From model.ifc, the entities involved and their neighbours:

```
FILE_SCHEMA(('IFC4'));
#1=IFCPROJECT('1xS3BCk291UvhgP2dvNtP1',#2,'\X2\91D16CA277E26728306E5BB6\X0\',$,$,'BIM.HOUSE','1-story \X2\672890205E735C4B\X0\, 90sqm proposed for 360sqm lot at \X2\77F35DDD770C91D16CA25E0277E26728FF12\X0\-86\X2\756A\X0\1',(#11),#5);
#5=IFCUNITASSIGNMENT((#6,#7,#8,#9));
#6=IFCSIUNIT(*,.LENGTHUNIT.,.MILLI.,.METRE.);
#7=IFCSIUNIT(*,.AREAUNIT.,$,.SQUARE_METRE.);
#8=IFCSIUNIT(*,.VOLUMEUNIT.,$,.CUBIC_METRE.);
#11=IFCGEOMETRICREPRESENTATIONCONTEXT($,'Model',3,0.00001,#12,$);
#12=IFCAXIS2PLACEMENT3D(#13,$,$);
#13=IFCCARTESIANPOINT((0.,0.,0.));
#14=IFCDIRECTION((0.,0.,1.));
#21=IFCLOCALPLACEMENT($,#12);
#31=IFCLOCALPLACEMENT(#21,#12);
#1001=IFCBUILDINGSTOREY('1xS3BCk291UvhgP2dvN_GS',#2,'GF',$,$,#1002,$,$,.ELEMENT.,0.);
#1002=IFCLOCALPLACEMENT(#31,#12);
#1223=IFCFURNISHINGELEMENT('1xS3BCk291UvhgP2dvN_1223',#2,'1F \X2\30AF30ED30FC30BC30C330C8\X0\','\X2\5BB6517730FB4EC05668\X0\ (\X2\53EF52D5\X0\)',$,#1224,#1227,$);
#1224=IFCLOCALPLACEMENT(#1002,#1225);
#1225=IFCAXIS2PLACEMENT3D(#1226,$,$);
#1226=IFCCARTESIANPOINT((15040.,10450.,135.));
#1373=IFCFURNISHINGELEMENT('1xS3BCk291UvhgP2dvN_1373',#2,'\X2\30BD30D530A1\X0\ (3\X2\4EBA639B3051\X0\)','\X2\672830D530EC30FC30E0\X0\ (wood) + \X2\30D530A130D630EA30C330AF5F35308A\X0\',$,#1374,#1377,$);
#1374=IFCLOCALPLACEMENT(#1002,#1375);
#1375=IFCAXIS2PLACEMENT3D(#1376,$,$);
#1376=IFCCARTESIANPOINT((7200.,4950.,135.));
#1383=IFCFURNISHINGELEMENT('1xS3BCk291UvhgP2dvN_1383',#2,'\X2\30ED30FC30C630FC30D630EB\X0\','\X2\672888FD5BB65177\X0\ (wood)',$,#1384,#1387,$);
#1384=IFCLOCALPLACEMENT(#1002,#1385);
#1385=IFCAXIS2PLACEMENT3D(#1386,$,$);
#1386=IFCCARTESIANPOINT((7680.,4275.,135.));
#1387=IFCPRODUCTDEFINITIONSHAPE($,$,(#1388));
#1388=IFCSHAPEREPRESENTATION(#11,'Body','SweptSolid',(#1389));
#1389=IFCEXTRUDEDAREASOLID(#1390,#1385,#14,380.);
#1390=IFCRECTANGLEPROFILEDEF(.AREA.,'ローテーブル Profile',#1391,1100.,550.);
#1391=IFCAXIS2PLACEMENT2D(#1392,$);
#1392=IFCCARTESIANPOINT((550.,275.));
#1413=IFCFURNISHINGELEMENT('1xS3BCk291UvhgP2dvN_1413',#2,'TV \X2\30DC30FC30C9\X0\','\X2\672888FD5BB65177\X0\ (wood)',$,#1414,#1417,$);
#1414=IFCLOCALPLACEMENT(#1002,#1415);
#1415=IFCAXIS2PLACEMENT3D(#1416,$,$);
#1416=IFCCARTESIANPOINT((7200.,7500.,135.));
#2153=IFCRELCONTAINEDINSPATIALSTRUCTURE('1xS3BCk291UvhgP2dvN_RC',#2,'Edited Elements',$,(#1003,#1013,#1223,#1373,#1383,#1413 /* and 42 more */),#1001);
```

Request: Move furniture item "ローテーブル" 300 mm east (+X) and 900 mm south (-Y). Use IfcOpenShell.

```python
import ifcopenshell
import ifcopenshell.api.geometry
import ifcopenshell.util.placement

model = ifcopenshell.open("model.ifc")

item = model.by_guid("1xS3BCk291UvhgP2dvN_1383")
matrix = ifcopenshell.util.placement.get_local_placement(item.ObjectPlacement)
matrix[0, 3] += 300.0
matrix[1, 3] -= 900.0
ifcopenshell.api.geometry.edit_object_placement(model, product=item, matrix=matrix, is_si=False)

print(ifcopenshell.util.placement.get_local_placement(item.ObjectPlacement).round(3) + 0.0)

model.write("model_v2.ifc")
```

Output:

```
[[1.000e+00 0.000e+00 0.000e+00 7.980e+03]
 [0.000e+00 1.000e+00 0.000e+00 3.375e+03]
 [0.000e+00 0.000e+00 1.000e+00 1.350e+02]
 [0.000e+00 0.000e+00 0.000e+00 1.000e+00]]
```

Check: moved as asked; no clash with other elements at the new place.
